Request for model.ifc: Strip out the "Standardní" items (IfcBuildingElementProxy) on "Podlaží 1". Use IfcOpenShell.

First a look at what the model holds.

```python
import ifcopenshell
import ifcopenshell.util.element

model = ifcopenshell.open("model.ifc")
print(model.schema)
storey = next(s for s in model.by_type("IfcBuildingStorey") if s.Name == "Podlaží 1")
proxies = [e for e in ifcopenshell.util.element.get_decomposition(storey) if e.is_a("IfcBuildingElementProxy")]
seen = {}
for e in proxies:
    element_type = ifcopenshell.util.element.get_type(e)
    name = element_type.Name if element_type not in (None, e) else None
    seen[name] = seen.get(name, 0) + 1
for name, count in sorted(seen.items(), key=str):
    print(count, "x", name)
```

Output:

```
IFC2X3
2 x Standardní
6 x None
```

```python
import ifcopenshell
import ifcopenshell.api.root
import ifcopenshell.util.element

model = ifcopenshell.open("model.ifc")

storey = next(s for s in model.by_type("IfcBuildingStorey") if s.Name == "Podlaží 1")
proxies = [e for e in ifcopenshell.util.element.get_decomposition(storey) if e.is_a("IfcBuildingElementProxy")]
targets = [e for e in proxies if (t := ifcopenshell.util.element.get_type(e)) not in (None, e) and t.Name == "Standardní"]

for e in targets:
    ifcopenshell.api.root.remove_product(model, product=e)
print(len(targets), "removed")

model.write("model_updated.ifc")
```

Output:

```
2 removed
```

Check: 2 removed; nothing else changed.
